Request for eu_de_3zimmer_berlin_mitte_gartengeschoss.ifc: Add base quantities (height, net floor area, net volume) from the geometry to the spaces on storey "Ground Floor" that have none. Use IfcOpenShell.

First a look at what the model holds.

```python
import ifcopenshell
import ifcopenshell.util.element
import ifcopenshell.util.unit

model = ifcopenshell.open("eu_de_3zimmer_berlin_mitte_gartengeschoss.ifc")
print(model.schema)
for unit_type in ("LENGTHUNIT", "AREAUNIT", "VOLUMEUNIT"):
    print(unit_type, ifcopenshell.util.unit.calculate_unit_scale(model, unit_type))
storey = next(s for s in model.by_type("IfcBuildingStorey") if s.Name == "Ground Floor")
spaces = [e for e in ifcopenshell.util.element.get_decomposition(storey) if e.is_a("IfcSpace")]
for e in sorted(spaces, key=lambda e: e.id()):
    print(e.id(), e.is_a(), e.Name, list(ifcopenshell.util.element.get_psets(e, qtos_only=True)), sep=" | ")
```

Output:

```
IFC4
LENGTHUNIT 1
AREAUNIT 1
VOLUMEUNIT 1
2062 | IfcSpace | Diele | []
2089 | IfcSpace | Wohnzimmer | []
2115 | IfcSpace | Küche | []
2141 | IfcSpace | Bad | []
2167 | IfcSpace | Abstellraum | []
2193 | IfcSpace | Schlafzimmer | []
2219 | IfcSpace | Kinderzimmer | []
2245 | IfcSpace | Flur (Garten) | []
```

```python
import ifcopenshell
import ifcopenshell.api.pset
import ifcopenshell.geom
import ifcopenshell.util.element
import ifcopenshell.util.shape
import ifcopenshell.util.unit

model = ifcopenshell.open("eu_de_3zimmer_berlin_mitte_gartengeschoss.ifc")
unit_scale = ifcopenshell.util.unit.calculate_unit_scale(model)
area_scale = ifcopenshell.util.unit.calculate_unit_scale(model, "AREAUNIT")
volume_scale = ifcopenshell.util.unit.calculate_unit_scale(model, "VOLUMEUNIT")
settings = ifcopenshell.geom.settings()

storey = next(s for s in model.by_type("IfcBuildingStorey") if s.Name == "Ground Floor")
spaces = [e for e in ifcopenshell.util.element.get_decomposition(storey) if e.is_a("IfcSpace")]

for e in sorted(spaces, key=lambda e: e.id()):
    if ifcopenshell.util.element.get_psets(e, qtos_only=True, should_inherit=False):
        continue
    # Geometry comes back in metres, in the element's own axes.
    shape = ifcopenshell.geom.create_shape(settings, e)
    values = {
        "Height": ifcopenshell.util.shape.get_z(shape.geometry) / unit_scale,
        "NetFloorArea": ifcopenshell.util.shape.get_footprint_area(shape.geometry) / area_scale,
        "NetVolume": ifcopenshell.util.shape.get_volume(shape.geometry) / volume_scale,
    }
    qto = ifcopenshell.api.pset.add_qto(model, product=e, name="Qto_SpaceBaseQuantities")
    ifcopenshell.api.pset.edit_qto(model, qto=qto, properties=values)
    print(e.id(), {k: round(v, 3) for k, v in values.items()})

model.write("eu_de_3zimmer_berlin_mitte_gartengeschoss-out.ifc")
```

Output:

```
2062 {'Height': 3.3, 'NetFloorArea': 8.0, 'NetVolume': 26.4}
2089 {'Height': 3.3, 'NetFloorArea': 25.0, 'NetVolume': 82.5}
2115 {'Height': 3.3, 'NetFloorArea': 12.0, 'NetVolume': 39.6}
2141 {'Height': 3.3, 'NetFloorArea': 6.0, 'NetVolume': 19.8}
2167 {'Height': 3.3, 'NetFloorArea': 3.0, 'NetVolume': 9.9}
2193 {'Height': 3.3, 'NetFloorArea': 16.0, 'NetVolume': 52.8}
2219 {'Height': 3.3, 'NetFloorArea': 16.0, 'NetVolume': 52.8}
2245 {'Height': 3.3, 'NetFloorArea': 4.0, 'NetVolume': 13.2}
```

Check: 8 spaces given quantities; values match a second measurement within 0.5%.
